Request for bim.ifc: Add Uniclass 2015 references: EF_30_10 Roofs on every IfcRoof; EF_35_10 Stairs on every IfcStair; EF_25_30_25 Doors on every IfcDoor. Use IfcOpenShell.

First a look at what the model holds.

```python
import ifcopenshell

model = ifcopenshell.open("bim.ifc")
print(model.schema)
print("classifications:", [c.Name for c in model.by_type("IfcClassification")])
for ifc_class in ("IfcDoor", "IfcRoof", "IfcStair", "IfcWall", "IfcWindow"):
    print(ifc_class, len(model.by_type(ifc_class)))
```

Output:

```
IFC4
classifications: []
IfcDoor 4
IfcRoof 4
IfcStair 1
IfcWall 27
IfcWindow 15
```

```python
import ifcopenshell
import ifcopenshell.api.classification

model = ifcopenshell.open("bim.ifc")

system = ifcopenshell.api.classification.add_classification(model, classification="Uniclass 2015")

codes = {
    "IfcRoof": ("EF_30_10", "Roofs"),
    "IfcStair": ("EF_35_10", "Stairs"),
    "IfcDoor": ("EF_25_30_25", "Doors"),
}
for ifc_class, (code, name) in codes.items():
    products = model.by_type(ifc_class)
    ifcopenshell.api.classification.add_reference(
        model, products=products, classification=system, identification=code, name=name
    )
    print(code, len(products))

model.write("bim_v2.ifc")
```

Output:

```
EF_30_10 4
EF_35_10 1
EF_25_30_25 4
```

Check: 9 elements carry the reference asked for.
